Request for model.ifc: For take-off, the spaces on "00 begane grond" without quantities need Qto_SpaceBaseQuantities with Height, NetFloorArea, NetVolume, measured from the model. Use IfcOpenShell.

First a look at what the model holds.

```python
import ifcopenshell
import ifcopenshell.util.element
import ifcopenshell.util.unit

model = ifcopenshell.open("model.ifc")
print(model.schema)
for unit_type in ("LENGTHUNIT", "AREAUNIT", "VOLUMEUNIT"):
    print(unit_type, ifcopenshell.util.unit.calculate_unit_scale(model, unit_type))
storey = next(s for s in model.by_type("IfcBuildingStorey") if s.Name == "00 begane grond")
spaces = [e for e in ifcopenshell.util.element.get_decomposition(storey) if e.is_a("IfcSpace")]
for e in sorted(spaces, key=lambda e: e.id()):
    print(e.id(), e.is_a(), e.Name, list(ifcopenshell.util.element.get_psets(e, qtos_only=True)), sep=" | ")
```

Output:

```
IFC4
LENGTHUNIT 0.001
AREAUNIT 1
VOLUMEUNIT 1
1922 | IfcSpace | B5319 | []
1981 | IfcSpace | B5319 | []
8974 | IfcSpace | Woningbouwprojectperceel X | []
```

```python
import ifcopenshell
import ifcopenshell.api.pset
import ifcopenshell.geom
import ifcopenshell.util.element
import ifcopenshell.util.shape
import ifcopenshell.util.unit

model = ifcopenshell.open("model.ifc")
unit_scale = ifcopenshell.util.unit.calculate_unit_scale(model)
area_scale = ifcopenshell.util.unit.calculate_unit_scale(model, "AREAUNIT")
volume_scale = ifcopenshell.util.unit.calculate_unit_scale(model, "VOLUMEUNIT")
settings = ifcopenshell.geom.settings()

storey = next(s for s in model.by_type("IfcBuildingStorey") if s.Name == "00 begane grond")
spaces = [e for e in ifcopenshell.util.element.get_decomposition(storey) if e.is_a("IfcSpace")]

for e in sorted(spaces, key=lambda e: e.id()):
    if ifcopenshell.util.element.get_psets(e, qtos_only=True, should_inherit=False):
        continue
    # Geometry comes back in metres, in the element's own axes.
    shape = ifcopenshell.geom.create_shape(settings, e)
    values = {
        "Height": ifcopenshell.util.shape.get_z(shape.geometry) / unit_scale,
        "NetFloorArea": ifcopenshell.util.shape.get_footprint_area(shape.geometry) / area_scale,
        "NetVolume": ifcopenshell.util.shape.get_volume(shape.geometry) / volume_scale,
    }
    qto = ifcopenshell.api.pset.add_qto(model, product=e, name="Qto_SpaceBaseQuantities")
    ifcopenshell.api.pset.edit_qto(model, qto=qto, properties=values)
    print(e.id(), {k: round(v, 3) for k, v in values.items()})

model.write("model_v2.ifc")
```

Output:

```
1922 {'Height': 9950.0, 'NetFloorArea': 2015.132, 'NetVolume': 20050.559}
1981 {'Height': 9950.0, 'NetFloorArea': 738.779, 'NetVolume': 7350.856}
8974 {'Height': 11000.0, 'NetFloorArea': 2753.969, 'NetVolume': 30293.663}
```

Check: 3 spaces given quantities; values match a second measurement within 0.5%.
